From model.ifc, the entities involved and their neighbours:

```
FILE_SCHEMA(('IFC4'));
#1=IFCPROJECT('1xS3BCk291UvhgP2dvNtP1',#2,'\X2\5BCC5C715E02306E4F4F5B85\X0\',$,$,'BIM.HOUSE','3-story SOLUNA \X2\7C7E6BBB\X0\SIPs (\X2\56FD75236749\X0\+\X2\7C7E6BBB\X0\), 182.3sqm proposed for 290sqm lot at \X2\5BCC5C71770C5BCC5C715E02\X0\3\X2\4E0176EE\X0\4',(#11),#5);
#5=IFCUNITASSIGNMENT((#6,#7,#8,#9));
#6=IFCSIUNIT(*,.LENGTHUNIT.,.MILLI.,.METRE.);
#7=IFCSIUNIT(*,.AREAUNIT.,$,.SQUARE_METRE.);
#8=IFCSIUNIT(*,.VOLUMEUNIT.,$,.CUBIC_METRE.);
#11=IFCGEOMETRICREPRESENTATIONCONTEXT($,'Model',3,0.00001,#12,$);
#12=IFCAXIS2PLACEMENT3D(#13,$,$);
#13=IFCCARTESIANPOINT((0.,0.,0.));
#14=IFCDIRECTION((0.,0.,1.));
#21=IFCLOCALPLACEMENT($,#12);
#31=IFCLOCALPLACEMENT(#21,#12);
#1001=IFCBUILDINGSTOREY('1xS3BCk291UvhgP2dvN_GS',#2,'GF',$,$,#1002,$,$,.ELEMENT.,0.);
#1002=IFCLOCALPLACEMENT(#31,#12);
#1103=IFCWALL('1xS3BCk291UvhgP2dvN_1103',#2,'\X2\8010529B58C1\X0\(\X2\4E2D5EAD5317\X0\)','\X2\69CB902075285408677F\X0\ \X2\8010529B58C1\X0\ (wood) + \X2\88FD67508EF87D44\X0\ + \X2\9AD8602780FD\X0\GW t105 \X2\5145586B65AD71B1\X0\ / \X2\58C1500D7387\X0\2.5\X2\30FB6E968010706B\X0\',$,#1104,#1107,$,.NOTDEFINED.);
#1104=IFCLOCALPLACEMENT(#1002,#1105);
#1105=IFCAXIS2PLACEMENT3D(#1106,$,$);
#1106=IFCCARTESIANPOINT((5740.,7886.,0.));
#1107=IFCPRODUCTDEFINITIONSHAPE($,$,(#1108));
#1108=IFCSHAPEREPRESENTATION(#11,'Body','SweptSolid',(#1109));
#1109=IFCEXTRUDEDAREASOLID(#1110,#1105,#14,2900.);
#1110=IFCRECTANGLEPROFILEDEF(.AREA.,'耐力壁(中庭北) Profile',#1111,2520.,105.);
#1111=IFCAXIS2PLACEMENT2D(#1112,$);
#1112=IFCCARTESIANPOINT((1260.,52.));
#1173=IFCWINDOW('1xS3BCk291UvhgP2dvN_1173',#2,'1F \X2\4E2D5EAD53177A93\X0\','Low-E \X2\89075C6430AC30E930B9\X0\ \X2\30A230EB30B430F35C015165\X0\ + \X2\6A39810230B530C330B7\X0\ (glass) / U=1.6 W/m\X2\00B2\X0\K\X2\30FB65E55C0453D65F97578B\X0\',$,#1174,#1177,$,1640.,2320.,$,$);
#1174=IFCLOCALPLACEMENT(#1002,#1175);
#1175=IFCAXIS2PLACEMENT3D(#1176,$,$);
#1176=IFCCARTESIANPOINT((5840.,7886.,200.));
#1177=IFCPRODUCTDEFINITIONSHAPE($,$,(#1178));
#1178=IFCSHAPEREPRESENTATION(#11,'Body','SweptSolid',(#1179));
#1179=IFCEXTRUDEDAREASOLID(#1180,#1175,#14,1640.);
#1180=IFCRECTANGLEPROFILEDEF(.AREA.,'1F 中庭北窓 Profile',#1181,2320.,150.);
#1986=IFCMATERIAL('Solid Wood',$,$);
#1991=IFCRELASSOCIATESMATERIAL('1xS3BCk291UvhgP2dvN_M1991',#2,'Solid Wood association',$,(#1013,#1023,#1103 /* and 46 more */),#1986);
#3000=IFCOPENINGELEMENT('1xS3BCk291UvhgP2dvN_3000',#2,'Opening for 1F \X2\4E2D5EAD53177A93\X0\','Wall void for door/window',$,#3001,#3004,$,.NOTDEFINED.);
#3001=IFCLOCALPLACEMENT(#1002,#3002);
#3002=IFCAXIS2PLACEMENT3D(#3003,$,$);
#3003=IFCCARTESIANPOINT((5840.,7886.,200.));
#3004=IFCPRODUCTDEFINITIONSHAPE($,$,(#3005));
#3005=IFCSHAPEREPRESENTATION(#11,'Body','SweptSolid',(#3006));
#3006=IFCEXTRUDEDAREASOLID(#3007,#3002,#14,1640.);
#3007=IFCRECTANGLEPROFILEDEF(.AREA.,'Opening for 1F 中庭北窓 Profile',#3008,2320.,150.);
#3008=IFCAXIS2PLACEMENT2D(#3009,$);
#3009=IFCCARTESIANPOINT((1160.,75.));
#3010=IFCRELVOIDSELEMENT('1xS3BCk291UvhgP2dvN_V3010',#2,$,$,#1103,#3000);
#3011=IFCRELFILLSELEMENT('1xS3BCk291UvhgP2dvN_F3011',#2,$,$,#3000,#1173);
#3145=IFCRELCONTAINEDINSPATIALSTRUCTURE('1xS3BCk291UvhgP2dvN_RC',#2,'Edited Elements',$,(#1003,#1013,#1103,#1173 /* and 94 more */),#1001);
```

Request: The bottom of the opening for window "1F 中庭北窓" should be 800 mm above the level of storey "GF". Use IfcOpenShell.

```python
import numpy as np
import ifcopenshell
import ifcopenshell.api.geometry
import ifcopenshell.geom
import ifcopenshell.util.element
import ifcopenshell.util.placement
import ifcopenshell.util.shape
import ifcopenshell.util.unit

model = ifcopenshell.open("model.ifc")
unit_scale = ifcopenshell.util.unit.calculate_unit_scale(model)

window = model.by_guid("1xS3BCk291UvhgP2dvN_1173")
opening = window.FillsVoids[0].RelatingOpeningElement
storey = ifcopenshell.util.element.get_container(window, ifc_class="IfcBuildingStorey")
level = ifcopenshell.util.placement.get_local_placement(storey.ObjectPlacement)[2, 3]

# The opening's origin need not be at the sill, so measure its lowest point.
shape = ifcopenshell.geom.create_shape(ifcopenshell.geom.settings(), opening)
bottom = ifcopenshell.util.shape.get_shape_bottom_elevation(shape, shape.geometry) / unit_scale
dz = level + 800.0 - bottom

shift = np.array([0.0, 0.0, dz])
# The window is not placed relative to its opening, so move both.
for product in (opening, window):
    matrix = ifcopenshell.util.placement.get_local_placement(product.ObjectPlacement)
    matrix[:3, 3] += shift
    ifcopenshell.api.geometry.edit_object_placement(model, product=product, matrix=matrix, is_si=False)

print(f"moved by {dz * unit_scale:+.3f} m")

model.write("model_rev.ifc")
```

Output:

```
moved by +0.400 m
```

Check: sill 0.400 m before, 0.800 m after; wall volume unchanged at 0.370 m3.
